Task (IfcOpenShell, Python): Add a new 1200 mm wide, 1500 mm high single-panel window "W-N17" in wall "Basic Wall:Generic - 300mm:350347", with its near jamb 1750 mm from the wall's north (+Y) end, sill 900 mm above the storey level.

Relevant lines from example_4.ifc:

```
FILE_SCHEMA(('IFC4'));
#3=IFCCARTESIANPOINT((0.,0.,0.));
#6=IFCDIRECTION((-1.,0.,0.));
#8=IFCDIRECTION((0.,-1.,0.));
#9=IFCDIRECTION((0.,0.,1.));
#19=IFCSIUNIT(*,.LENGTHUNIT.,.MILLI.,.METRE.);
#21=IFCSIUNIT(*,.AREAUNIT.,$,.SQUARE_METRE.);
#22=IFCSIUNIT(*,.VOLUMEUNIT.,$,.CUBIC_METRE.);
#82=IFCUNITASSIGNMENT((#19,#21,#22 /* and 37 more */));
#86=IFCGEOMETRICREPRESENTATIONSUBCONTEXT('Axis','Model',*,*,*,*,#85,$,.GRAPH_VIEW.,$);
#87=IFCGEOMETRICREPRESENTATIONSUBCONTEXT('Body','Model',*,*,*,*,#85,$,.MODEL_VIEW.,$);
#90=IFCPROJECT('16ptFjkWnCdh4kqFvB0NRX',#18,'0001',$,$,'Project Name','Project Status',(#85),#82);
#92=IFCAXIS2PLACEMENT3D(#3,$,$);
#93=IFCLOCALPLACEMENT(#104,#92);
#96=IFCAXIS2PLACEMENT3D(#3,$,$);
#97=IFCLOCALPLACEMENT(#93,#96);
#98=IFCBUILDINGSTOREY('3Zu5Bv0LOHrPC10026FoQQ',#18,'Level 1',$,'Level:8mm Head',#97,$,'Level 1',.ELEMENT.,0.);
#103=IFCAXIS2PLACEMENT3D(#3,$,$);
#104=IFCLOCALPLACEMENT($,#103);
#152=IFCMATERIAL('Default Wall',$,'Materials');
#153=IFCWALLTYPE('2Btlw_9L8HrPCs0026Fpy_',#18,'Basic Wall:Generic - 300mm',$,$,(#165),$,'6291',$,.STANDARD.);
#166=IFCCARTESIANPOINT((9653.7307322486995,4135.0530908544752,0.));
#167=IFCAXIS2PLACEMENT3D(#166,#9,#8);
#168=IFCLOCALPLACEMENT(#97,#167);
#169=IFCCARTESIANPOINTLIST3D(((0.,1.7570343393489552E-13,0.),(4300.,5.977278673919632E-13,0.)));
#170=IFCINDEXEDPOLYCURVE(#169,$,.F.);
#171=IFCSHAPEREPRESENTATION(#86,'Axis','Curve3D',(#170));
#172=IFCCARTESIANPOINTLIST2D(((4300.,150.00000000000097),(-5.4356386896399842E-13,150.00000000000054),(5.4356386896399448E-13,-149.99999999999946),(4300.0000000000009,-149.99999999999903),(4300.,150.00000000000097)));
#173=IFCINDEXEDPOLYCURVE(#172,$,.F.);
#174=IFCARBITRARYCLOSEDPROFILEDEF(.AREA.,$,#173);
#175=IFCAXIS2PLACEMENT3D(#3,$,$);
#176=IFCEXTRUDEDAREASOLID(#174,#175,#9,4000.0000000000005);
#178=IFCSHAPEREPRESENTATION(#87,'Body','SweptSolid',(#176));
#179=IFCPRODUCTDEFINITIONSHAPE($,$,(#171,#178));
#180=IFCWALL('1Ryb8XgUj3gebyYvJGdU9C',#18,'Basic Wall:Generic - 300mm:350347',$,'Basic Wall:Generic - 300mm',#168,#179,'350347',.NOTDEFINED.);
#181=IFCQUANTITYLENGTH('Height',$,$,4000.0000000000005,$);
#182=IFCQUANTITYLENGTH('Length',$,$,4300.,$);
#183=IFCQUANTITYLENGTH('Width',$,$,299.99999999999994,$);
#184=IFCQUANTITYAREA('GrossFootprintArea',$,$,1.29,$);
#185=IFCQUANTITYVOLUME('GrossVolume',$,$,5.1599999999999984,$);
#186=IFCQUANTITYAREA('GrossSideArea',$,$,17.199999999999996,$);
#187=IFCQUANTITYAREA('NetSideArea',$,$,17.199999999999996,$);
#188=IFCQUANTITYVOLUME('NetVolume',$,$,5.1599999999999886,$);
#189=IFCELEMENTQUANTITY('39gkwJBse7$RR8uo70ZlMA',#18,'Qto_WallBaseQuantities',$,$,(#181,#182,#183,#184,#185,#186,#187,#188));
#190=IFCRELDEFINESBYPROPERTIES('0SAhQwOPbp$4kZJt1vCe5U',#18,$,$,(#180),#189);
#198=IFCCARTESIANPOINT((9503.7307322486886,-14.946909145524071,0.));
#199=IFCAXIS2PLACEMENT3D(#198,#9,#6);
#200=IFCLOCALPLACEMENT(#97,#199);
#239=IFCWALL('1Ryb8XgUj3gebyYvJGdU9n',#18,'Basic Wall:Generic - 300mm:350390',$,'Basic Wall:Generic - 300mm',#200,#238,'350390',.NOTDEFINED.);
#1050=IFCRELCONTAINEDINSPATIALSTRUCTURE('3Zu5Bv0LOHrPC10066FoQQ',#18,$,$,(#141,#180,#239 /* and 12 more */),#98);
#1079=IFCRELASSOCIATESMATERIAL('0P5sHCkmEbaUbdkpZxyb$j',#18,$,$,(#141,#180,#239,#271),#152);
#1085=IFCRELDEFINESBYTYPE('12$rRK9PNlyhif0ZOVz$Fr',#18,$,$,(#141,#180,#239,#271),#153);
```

```python
import numpy as np
import ifcopenshell
import ifcopenshell.api.feature
import ifcopenshell.api.geometry
import ifcopenshell.api.pset
import ifcopenshell.api.root
import ifcopenshell.api.spatial
import ifcopenshell.geom
import ifcopenshell.util.element
import ifcopenshell.util.placement
import ifcopenshell.util.representation
import ifcopenshell.util.shape
import ifcopenshell.util.unit

model = ifcopenshell.open("example_4.ifc")
unit_scale = ifcopenshell.util.unit.calculate_unit_scale(model)
area_scale = ifcopenshell.util.unit.calculate_unit_scale(model, "AREAUNIT")
volume_scale = ifcopenshell.util.unit.calculate_unit_scale(model, "VOLUMEUNIT")
settings = ifcopenshell.geom.settings()


def volume(element):
    """Net volume in cubic metres, openings subtracted."""
    shape = ifcopenshell.geom.create_shape(settings, element)
    return ifcopenshell.util.shape.get_volume(shape.geometry)


wall = model.by_guid("1Ryb8XgUj3gebyYvJGdU9C")
storey = ifcopenshell.util.element.get_container(wall, ifc_class="IfcBuildingStorey")
context = ifcopenshell.util.representation.get_context(model, "Model", "Body", "MODEL_VIEW")
before = volume(wall)

width, height, from_end, sill = 1.2, 1.5, 1.75, 0.9  # metres

# The wall runs along its own X axis, and the end named is its -X end.
wall_shape = ifcopenshell.geom.create_shape(settings, wall)
x, y, z = ifcopenshell.util.shape.get_vertices(wall_shape.geometry).T
start = x.min() + from_end
face, thickness = float(y.min()), float(y.max() - y.min())
wall_matrix = ifcopenshell.util.placement.get_local_placement(wall.ObjectPlacement)
level = ifcopenshell.util.placement.get_local_placement(storey.ObjectPlacement)[2, 3]


def in_wall(x, y):
    """Placement at x, y metres in the wall's axes, at sill height."""
    matrix = wall_matrix.copy()
    matrix[:, 3] = wall_matrix @ np.array([x / unit_scale, y / unit_scale, 0.0, 1.0])
    matrix[2, 3] = level + sill / unit_scale
    return matrix


# Opening: a box that overshoots both wall faces by 50 mm.
opening = ifcopenshell.api.root.create_entity(model, ifc_class="IfcOpeningElement", predefined_type="OPENING")
box = ifcopenshell.api.geometry.add_wall_representation(
    model, context=context, length=width, height=height, thickness=thickness + 0.1
)
ifcopenshell.api.geometry.assign_representation(model, product=opening, representation=box)
ifcopenshell.api.geometry.edit_object_placement(model, product=opening, matrix=in_wall(start, face - 0.05), is_si=False)
ifcopenshell.api.feature.add_feature(model, feature=opening, element=wall)

window = ifcopenshell.api.root.create_entity(model, ifc_class="IfcWindow", name="W-N17", predefined_type="WINDOW")
window.OverallWidth, window.OverallHeight = width / unit_scale, height / unit_scale
window.PartitioningType = "SINGLE_PANEL"
body = ifcopenshell.api.geometry.add_window_representation(
    model,
    context=context,
    overall_width=window.OverallWidth,
    overall_height=window.OverallHeight,
    partition_type="SINGLE_PANEL",
)
ifcopenshell.api.geometry.assign_representation(model, product=window, representation=body)
ifcopenshell.api.spatial.assign_container(model, products=[window], relating_structure=storey)
ifcopenshell.api.feature.add_filling(model, opening=opening, element=window)

# Centre the window in the wall's thickness.
ifcopenshell.api.geometry.edit_object_placement(model, product=window, matrix=in_wall(start, face), is_si=False)
window_shape = ifcopenshell.geom.create_shape(settings, window)
depth = ifcopenshell.util.shape.get_vertices(window_shape.geometry)[:, 1]
offset = face + thickness / 2 - (depth.min() + depth.max()) / 2
ifcopenshell.api.geometry.edit_object_placement(model, product=window, matrix=in_wall(start, offset), is_si=False)

after = volume(wall)

# Update the wall's stored quantities.
qto = model.by_id(ifcopenshell.util.element.get_pset(wall, "Qto_WallBaseQuantities", should_inherit=False)["id"])
ifcopenshell.api.pset.edit_qto(model, qto=qto, properties={
    "NetSideArea": after / thickness / area_scale,
    "NetVolume": after / volume_scale,
})

print(f"wall volume {before:.3f} -> {after:.3f} m3")

model.write("example_4-out.ifc")
```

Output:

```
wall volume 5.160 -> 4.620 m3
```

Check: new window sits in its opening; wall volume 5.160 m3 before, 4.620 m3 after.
